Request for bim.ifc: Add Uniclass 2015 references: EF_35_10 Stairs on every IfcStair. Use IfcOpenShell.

First a look at what the model holds.

```python
import ifcopenshell

model = ifcopenshell.open("bim.ifc")
print(model.schema)
print("classifications:", [c.Name for c in model.by_type("IfcClassification")])
for ifc_class in ("IfcDoor", "IfcRoof", "IfcStair", "IfcWall", "IfcWindow"):
    print(ifc_class, len(model.by_type(ifc_class)))
```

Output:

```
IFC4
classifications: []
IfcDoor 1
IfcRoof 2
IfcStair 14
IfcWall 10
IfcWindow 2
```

```python
import ifcopenshell
import ifcopenshell.api.classification

model = ifcopenshell.open("bim.ifc")

system = ifcopenshell.api.classification.add_classification(model, classification="Uniclass 2015")

codes = {
    "IfcStair": ("EF_35_10", "Stairs"),
}
for ifc_class, (code, name) in codes.items():
    products = model.by_type(ifc_class)
    ifcopenshell.api.classification.add_reference(
        model, products=products, classification=system, identification=code, name=name
    )
    print(code, len(products))

model.write("bim_edited.ifc")
```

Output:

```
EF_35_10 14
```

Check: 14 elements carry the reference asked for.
